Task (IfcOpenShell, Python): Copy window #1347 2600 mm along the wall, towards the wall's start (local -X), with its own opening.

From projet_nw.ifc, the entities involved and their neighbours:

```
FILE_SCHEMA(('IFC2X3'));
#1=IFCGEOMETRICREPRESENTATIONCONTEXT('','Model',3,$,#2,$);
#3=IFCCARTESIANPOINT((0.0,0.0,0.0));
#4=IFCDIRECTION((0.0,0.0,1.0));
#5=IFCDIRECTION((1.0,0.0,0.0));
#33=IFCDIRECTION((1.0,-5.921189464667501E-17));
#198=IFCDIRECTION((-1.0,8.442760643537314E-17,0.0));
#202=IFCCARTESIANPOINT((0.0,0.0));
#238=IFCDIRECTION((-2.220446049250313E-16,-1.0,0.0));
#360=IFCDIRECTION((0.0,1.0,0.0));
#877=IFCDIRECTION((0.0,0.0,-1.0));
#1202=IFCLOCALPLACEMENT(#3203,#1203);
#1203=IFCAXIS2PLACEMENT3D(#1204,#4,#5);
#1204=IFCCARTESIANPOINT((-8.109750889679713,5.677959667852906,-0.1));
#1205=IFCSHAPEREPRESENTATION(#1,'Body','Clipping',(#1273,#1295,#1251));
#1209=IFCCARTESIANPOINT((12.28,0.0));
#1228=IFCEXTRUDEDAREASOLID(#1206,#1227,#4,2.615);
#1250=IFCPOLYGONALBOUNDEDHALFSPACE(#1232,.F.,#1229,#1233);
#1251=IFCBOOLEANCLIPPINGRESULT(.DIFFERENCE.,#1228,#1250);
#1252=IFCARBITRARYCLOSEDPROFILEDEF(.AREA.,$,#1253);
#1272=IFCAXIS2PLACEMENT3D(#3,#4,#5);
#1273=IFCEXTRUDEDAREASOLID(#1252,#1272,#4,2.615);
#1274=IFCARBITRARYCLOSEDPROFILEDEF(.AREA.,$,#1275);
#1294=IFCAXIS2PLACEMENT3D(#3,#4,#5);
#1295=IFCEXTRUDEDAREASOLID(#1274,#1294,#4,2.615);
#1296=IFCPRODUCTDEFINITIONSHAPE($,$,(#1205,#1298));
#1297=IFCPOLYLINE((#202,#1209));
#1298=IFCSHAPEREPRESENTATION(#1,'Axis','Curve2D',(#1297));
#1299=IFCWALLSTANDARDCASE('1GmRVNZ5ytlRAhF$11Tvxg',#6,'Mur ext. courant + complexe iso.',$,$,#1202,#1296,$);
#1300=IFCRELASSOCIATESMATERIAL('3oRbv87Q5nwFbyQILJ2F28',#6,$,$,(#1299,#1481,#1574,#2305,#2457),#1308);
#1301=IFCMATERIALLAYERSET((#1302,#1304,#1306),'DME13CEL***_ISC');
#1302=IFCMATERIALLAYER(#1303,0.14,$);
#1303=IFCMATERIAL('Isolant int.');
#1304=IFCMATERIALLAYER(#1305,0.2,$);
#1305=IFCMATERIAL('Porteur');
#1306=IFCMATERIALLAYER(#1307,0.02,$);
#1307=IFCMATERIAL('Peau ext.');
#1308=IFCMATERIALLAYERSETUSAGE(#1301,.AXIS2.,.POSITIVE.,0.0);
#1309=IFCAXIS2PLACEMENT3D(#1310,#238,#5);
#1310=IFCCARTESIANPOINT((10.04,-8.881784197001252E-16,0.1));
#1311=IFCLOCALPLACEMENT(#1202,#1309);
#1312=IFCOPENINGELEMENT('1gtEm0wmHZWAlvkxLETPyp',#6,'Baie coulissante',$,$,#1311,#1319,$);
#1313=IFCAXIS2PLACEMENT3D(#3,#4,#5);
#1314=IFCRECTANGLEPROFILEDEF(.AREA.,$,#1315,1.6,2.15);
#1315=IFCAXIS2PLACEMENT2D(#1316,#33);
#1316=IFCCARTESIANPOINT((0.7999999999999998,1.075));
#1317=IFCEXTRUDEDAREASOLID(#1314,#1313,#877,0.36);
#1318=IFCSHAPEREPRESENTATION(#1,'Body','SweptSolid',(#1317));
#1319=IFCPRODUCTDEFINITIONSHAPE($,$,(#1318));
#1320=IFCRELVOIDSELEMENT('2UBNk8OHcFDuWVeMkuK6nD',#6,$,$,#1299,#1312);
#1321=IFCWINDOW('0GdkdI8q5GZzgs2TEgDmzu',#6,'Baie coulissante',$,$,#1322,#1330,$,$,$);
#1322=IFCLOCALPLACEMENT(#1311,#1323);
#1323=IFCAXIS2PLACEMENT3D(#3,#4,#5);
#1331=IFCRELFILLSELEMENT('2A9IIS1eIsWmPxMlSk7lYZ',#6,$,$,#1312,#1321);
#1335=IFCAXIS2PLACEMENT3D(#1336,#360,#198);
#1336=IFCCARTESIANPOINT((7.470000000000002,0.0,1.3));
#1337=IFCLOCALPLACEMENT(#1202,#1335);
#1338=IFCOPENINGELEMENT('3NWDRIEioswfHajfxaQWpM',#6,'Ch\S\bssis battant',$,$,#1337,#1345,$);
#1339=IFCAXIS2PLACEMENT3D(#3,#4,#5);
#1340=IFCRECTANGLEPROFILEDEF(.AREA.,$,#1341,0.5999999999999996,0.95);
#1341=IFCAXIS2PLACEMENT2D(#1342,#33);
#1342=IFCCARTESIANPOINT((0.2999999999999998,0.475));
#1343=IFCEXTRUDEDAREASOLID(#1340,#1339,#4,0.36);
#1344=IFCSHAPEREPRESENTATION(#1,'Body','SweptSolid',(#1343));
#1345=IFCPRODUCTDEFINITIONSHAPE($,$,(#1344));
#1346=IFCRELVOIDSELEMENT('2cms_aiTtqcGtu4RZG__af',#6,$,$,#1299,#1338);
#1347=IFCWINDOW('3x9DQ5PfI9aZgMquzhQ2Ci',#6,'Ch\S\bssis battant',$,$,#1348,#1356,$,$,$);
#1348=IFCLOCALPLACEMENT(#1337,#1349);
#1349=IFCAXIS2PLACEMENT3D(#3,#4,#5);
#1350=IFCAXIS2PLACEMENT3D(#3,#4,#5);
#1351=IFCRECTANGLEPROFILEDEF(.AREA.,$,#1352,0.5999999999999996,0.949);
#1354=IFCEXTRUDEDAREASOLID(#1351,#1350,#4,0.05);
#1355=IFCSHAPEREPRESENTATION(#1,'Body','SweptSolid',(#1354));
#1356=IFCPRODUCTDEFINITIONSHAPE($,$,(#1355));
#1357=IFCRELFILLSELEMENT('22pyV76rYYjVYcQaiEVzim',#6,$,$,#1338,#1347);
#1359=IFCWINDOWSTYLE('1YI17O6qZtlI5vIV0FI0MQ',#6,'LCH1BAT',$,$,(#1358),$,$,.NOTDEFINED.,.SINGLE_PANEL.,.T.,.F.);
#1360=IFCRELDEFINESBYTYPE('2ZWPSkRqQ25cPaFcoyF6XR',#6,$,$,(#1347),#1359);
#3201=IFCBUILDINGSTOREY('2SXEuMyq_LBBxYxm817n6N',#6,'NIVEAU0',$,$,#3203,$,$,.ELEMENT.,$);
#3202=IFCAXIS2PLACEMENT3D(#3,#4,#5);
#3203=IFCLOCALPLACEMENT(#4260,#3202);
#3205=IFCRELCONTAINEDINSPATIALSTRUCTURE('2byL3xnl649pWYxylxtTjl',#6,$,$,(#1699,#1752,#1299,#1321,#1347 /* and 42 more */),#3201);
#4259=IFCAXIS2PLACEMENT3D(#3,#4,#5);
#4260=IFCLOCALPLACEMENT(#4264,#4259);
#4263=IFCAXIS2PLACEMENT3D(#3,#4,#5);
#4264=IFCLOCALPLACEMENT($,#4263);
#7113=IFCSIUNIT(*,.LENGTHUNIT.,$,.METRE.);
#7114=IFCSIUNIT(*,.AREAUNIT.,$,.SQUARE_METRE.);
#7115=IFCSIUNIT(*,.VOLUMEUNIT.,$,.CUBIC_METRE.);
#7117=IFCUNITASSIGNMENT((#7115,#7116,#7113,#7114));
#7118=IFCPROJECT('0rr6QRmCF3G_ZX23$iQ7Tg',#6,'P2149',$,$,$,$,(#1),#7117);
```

```python
import ifcopenshell
import ifcopenshell.api.feature
import ifcopenshell.api.geometry
import ifcopenshell.api.root
import ifcopenshell.geom
import ifcopenshell.util.element
import ifcopenshell.util.placement
import ifcopenshell.util.shape

model = ifcopenshell.open("projet_nw.ifc")
settings = ifcopenshell.geom.settings()


def volume(element):
    """Net volume in cubic metres, openings subtracted."""
    shape = ifcopenshell.geom.create_shape(settings, element)
    return ifcopenshell.util.shape.get_volume(shape.geometry)


window = model.by_guid("3x9DQ5PfI9aZgMquzhQ2Ci")
opening = window.FillsVoids[0].RelatingOpeningElement
wall = opening.VoidsElements[0].RelatingBuildingElement
before = volume(wall)
shift = ifcopenshell.util.placement.get_local_placement(wall.ObjectPlacement)[:3, 0] * -2.6

# copy_class copies the void relationship, type, container and properties, but no geometry.
new_opening = ifcopenshell.api.root.copy_class(model, product=opening)
new_opening.Representation = ifcopenshell.util.element.copy_deep(
    model, opening.Representation, exclude=["IfcGeometricRepresentationContext", "IfcRepresentationMap"]
)
new_window = ifcopenshell.api.root.copy_class(model, product=window)
new_window.Representation = ifcopenshell.util.element.copy_deep(
    model, window.Representation, exclude=["IfcGeometricRepresentationContext", "IfcRepresentationMap"]
)
fills = ifcopenshell.api.feature.add_filling(model, opening=new_opening, element=new_window)
fills.OwnerHistory = new_window.OwnerHistory  # required in IFC2X3

for old, new in ((opening, new_opening), (window, new_window)):
    matrix = ifcopenshell.util.placement.get_local_placement(old.ObjectPlacement)
    matrix[:3, 3] += shift
    ifcopenshell.api.geometry.edit_object_placement(model, product=new, matrix=matrix, is_si=False)

after = volume(wall)

print(f"wall volume {before:.3f} -> {after:.3f} m3")

model.write("projet_nw_rev.ifc")
```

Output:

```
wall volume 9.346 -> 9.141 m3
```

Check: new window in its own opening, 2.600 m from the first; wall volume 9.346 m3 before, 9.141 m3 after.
